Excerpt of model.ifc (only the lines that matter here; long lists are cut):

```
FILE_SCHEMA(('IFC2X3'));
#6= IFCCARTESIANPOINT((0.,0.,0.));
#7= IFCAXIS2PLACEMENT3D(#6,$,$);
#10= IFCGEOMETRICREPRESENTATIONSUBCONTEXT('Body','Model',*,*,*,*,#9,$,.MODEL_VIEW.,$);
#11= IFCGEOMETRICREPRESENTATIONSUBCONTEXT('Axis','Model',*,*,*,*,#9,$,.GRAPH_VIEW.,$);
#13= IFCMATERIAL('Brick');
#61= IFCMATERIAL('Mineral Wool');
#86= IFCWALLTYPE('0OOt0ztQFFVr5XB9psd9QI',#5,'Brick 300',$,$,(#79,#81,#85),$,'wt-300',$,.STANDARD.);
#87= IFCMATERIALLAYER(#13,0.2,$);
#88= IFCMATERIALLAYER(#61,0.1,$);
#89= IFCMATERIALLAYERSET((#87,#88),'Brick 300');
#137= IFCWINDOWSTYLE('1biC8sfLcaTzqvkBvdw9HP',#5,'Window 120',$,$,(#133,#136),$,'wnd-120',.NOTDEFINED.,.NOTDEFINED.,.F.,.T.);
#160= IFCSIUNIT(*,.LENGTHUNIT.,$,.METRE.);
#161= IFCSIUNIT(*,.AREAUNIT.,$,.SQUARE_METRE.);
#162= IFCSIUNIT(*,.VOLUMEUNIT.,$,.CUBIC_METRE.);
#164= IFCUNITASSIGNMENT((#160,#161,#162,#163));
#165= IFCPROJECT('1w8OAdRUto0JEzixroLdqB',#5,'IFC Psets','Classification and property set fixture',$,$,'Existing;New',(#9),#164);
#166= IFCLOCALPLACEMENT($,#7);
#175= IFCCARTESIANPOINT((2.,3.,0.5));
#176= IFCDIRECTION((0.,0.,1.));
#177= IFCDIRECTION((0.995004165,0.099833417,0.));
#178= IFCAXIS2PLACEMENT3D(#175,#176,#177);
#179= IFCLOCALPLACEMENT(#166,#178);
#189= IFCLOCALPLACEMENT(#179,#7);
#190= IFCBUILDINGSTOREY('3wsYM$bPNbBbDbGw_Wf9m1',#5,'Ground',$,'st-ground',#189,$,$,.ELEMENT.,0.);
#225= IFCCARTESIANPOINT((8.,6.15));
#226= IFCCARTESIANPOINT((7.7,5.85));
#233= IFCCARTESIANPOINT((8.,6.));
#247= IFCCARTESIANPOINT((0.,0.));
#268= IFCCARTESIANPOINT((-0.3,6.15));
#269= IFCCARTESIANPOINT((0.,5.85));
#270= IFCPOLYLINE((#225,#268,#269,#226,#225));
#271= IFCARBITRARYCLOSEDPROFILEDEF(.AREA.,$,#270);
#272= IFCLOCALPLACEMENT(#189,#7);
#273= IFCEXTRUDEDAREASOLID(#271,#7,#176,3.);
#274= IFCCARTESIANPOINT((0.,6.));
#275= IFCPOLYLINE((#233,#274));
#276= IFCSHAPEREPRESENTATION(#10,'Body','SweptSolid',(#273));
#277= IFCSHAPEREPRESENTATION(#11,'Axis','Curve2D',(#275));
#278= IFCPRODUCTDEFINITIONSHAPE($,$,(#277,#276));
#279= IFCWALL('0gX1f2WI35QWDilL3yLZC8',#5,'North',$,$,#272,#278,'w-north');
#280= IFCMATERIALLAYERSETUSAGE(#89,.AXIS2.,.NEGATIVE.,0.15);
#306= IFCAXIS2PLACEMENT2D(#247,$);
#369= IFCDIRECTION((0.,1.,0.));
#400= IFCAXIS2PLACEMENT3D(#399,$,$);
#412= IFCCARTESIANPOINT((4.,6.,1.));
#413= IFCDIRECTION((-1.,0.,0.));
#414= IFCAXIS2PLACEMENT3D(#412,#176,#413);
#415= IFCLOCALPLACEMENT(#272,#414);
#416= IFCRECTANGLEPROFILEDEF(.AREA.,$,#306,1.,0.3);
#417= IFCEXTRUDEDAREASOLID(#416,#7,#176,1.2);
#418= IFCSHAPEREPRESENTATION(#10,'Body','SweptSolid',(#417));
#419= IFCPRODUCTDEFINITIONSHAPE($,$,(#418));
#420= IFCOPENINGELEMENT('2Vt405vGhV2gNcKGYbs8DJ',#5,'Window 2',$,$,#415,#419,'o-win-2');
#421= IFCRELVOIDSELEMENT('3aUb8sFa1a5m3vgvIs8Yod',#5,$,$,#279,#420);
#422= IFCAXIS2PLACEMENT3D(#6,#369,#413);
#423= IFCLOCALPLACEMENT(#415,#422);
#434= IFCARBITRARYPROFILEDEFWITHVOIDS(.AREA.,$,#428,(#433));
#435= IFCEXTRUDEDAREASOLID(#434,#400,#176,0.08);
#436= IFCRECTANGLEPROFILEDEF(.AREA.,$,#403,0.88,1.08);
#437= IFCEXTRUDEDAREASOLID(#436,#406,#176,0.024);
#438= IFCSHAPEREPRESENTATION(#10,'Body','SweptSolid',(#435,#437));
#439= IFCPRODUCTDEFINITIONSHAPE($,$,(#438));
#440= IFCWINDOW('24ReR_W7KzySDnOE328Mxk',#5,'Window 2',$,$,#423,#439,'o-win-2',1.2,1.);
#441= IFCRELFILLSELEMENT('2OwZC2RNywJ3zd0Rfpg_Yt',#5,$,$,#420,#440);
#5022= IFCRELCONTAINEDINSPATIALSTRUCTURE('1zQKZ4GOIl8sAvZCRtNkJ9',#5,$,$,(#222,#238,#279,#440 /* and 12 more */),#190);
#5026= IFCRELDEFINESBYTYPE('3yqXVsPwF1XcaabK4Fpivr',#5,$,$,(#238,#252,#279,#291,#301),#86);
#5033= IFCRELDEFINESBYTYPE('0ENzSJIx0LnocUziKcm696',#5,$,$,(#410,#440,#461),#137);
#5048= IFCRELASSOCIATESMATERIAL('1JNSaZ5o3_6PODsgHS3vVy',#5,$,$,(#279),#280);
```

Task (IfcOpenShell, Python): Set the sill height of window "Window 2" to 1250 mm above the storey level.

```python
import numpy as np
import ifcopenshell
import ifcopenshell.api.geometry
import ifcopenshell.geom
import ifcopenshell.util.element
import ifcopenshell.util.placement
import ifcopenshell.util.shape
import ifcopenshell.util.unit

model = ifcopenshell.open("model.ifc")
unit_scale = ifcopenshell.util.unit.calculate_unit_scale(model)

window = model.by_guid("24ReR_W7KzySDnOE328Mxk")
opening = window.FillsVoids[0].RelatingOpeningElement
storey = ifcopenshell.util.element.get_container(window, ifc_class="IfcBuildingStorey")
level = ifcopenshell.util.placement.get_local_placement(storey.ObjectPlacement)[2, 3]

# The opening's origin need not be at the sill, so measure its lowest point.
shape = ifcopenshell.geom.create_shape(ifcopenshell.geom.settings(), opening)
bottom = ifcopenshell.util.shape.get_shape_bottom_elevation(shape, shape.geometry) / unit_scale
dz = level + 1.25 / unit_scale - bottom

shift = np.array([0.0, 0.0, dz])
# The window is placed relative to its opening, so it follows when the opening moves.
matrix = ifcopenshell.util.placement.get_local_placement(opening.ObjectPlacement)
matrix[:3, 3] += shift
ifcopenshell.api.geometry.edit_object_placement(
    model, product=opening, matrix=matrix, is_si=False, should_transform_children=True
)

print(f"moved by {dz * unit_scale:+.3f} m")

model.write("model-out.ifc")
```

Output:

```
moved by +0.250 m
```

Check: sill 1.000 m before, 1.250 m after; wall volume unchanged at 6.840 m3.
